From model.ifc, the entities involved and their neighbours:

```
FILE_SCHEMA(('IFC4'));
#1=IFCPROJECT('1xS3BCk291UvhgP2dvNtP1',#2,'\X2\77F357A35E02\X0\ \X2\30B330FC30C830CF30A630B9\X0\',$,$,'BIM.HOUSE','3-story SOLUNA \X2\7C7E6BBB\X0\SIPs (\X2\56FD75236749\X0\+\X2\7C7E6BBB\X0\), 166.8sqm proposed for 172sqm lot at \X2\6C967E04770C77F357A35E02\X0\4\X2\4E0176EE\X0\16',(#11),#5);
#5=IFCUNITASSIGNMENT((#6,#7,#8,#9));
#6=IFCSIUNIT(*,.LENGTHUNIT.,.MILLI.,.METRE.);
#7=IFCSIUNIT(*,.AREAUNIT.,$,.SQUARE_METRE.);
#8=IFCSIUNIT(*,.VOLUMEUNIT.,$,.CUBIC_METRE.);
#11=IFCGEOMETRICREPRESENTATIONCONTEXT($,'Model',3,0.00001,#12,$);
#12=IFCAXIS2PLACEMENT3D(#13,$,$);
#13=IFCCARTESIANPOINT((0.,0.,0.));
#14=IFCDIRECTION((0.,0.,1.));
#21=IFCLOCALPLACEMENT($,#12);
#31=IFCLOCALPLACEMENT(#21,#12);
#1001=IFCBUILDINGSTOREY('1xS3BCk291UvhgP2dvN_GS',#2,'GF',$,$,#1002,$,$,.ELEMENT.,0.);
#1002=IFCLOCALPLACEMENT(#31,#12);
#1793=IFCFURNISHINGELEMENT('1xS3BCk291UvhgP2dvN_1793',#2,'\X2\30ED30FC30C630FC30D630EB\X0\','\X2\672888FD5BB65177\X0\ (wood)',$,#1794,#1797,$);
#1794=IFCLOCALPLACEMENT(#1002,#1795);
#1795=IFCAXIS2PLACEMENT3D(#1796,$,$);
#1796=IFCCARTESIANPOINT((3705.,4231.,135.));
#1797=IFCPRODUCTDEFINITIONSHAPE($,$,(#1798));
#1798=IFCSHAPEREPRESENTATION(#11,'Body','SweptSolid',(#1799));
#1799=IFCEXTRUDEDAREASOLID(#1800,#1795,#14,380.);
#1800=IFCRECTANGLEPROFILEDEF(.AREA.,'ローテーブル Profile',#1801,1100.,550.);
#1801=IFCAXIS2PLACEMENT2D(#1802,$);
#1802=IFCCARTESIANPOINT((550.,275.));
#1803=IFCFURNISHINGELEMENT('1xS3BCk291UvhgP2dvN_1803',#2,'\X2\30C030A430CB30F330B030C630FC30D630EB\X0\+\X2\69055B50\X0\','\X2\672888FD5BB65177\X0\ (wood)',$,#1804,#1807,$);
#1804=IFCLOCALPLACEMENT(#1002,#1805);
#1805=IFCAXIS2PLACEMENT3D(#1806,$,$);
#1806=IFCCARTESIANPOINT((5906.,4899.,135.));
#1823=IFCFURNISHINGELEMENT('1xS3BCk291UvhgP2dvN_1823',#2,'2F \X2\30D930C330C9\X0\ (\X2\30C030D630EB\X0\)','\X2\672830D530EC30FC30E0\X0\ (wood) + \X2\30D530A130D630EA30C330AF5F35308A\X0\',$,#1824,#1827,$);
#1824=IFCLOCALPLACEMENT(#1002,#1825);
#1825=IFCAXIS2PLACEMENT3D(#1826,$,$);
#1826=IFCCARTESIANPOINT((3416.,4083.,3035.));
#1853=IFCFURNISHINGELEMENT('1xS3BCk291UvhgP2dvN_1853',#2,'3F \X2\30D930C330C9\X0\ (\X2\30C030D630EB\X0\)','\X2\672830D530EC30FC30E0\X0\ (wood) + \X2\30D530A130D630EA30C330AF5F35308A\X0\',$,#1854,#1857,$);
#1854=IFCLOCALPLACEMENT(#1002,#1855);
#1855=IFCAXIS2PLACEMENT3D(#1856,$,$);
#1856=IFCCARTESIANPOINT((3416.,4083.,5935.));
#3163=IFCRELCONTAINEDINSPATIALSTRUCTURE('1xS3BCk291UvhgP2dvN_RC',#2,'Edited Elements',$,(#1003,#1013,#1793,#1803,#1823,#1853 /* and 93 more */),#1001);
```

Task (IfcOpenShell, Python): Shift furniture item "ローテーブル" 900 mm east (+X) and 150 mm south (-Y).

```python
import ifcopenshell
import ifcopenshell.api.geometry
import ifcopenshell.util.placement

model = ifcopenshell.open("model.ifc")

item = model.by_id(1793)
matrix = ifcopenshell.util.placement.get_local_placement(item.ObjectPlacement)
matrix[0, 3] += 900.0
matrix[1, 3] -= 150.0
ifcopenshell.api.geometry.edit_object_placement(model, product=item, matrix=matrix, is_si=False)

print(ifcopenshell.util.placement.get_local_placement(item.ObjectPlacement).round(3) + 0.0)

model.write("model_v2.ifc")
```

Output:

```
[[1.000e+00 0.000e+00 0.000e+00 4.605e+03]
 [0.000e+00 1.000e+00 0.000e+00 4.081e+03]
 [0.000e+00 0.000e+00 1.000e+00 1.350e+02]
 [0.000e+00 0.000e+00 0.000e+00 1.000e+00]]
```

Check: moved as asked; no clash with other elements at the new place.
